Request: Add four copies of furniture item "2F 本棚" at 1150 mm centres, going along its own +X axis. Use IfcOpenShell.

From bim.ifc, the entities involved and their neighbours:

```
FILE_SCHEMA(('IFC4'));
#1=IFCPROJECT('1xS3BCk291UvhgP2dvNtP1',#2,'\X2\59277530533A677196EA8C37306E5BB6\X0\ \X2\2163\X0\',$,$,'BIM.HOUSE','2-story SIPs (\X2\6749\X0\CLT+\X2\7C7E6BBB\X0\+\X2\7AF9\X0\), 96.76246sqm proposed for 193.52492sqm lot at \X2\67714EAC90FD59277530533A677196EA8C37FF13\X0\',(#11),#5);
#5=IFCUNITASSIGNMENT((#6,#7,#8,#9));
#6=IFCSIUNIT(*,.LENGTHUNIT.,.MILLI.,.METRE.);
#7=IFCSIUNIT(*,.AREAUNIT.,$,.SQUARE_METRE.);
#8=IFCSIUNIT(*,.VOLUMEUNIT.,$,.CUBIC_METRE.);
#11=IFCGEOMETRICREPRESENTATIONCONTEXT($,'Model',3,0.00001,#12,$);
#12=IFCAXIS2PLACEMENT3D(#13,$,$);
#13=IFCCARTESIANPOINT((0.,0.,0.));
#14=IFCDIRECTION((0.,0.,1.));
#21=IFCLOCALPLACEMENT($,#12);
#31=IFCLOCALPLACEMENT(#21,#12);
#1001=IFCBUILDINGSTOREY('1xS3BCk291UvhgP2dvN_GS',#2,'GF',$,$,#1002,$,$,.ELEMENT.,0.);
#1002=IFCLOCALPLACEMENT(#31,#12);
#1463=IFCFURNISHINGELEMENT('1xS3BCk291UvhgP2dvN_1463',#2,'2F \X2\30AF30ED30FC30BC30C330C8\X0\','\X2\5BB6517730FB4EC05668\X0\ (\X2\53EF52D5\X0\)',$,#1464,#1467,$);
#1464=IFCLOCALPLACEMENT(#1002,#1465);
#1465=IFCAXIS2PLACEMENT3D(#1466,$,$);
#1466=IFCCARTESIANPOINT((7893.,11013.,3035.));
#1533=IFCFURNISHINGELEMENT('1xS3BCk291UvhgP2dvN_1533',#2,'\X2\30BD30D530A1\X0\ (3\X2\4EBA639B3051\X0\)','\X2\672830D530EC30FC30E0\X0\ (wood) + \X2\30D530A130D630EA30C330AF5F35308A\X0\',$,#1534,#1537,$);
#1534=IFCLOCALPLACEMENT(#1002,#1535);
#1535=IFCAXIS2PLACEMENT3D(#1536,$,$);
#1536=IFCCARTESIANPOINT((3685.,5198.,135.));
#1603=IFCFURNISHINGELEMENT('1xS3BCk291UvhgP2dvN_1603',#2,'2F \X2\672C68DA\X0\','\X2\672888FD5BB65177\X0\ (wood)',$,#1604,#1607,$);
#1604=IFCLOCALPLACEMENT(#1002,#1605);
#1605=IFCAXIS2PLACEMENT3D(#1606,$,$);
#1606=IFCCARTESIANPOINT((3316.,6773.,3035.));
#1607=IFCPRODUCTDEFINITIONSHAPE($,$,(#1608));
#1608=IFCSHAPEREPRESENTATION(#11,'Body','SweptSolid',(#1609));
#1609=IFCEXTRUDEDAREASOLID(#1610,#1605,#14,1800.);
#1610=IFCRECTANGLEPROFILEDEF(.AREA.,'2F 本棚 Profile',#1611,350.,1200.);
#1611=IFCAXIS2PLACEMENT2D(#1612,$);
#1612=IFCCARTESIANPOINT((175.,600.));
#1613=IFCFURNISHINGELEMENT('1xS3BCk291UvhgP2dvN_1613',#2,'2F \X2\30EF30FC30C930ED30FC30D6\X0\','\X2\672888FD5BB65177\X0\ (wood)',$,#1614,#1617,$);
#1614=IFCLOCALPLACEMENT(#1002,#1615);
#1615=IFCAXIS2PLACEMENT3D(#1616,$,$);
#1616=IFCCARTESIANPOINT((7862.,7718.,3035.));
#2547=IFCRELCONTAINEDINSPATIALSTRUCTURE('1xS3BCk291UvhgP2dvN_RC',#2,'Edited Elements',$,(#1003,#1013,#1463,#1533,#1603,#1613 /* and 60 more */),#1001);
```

```python
import ifcopenshell
import ifcopenshell.api.geometry
import ifcopenshell.api.root
import ifcopenshell.util.element
import ifcopenshell.util.placement
import ifcopenshell.util.unit

model = ifcopenshell.open("bim.ifc")
unit_scale = ifcopenshell.util.unit.calculate_unit_scale(model)


def reuse_history(source, copy):
    """copy_class also copies each property set's owner history, people and application; keep the originals."""
    for rel in copy.IsDefinedBy:
        if rel.is_a("IfcRelDefinesByProperties") and (history := rel.RelatingPropertyDefinition.OwnerHistory):
            rel.RelatingPropertyDefinition.OwnerHistory = source.OwnerHistory
            ifcopenshell.util.element.remove_deep2(model, history)


source = model.by_id(1603)
base = ifcopenshell.util.placement.get_local_placement(source.ObjectPlacement)
step = base[:3, 0] * 1.15 / unit_scale

for i in range(1, 5):
    copy = ifcopenshell.api.root.copy_class(model, product=source)
    copy.Representation = ifcopenshell.util.element.copy_deep(
        model, source.Representation, exclude=["IfcGeometricRepresentationContext", "IfcRepresentationMap"]
    )
    reuse_history(source, copy)
    matrix = base.copy()
    matrix[:3, 3] += i * step
    print("added at", matrix[:3, 3].round(3) + 0.0)
    ifcopenshell.api.geometry.edit_object_placement(model, product=copy, matrix=matrix, is_si=False)

model.write("bim_edited.ifc")
```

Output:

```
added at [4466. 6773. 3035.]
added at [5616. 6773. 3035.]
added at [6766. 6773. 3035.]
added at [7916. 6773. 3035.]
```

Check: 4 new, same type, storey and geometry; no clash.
